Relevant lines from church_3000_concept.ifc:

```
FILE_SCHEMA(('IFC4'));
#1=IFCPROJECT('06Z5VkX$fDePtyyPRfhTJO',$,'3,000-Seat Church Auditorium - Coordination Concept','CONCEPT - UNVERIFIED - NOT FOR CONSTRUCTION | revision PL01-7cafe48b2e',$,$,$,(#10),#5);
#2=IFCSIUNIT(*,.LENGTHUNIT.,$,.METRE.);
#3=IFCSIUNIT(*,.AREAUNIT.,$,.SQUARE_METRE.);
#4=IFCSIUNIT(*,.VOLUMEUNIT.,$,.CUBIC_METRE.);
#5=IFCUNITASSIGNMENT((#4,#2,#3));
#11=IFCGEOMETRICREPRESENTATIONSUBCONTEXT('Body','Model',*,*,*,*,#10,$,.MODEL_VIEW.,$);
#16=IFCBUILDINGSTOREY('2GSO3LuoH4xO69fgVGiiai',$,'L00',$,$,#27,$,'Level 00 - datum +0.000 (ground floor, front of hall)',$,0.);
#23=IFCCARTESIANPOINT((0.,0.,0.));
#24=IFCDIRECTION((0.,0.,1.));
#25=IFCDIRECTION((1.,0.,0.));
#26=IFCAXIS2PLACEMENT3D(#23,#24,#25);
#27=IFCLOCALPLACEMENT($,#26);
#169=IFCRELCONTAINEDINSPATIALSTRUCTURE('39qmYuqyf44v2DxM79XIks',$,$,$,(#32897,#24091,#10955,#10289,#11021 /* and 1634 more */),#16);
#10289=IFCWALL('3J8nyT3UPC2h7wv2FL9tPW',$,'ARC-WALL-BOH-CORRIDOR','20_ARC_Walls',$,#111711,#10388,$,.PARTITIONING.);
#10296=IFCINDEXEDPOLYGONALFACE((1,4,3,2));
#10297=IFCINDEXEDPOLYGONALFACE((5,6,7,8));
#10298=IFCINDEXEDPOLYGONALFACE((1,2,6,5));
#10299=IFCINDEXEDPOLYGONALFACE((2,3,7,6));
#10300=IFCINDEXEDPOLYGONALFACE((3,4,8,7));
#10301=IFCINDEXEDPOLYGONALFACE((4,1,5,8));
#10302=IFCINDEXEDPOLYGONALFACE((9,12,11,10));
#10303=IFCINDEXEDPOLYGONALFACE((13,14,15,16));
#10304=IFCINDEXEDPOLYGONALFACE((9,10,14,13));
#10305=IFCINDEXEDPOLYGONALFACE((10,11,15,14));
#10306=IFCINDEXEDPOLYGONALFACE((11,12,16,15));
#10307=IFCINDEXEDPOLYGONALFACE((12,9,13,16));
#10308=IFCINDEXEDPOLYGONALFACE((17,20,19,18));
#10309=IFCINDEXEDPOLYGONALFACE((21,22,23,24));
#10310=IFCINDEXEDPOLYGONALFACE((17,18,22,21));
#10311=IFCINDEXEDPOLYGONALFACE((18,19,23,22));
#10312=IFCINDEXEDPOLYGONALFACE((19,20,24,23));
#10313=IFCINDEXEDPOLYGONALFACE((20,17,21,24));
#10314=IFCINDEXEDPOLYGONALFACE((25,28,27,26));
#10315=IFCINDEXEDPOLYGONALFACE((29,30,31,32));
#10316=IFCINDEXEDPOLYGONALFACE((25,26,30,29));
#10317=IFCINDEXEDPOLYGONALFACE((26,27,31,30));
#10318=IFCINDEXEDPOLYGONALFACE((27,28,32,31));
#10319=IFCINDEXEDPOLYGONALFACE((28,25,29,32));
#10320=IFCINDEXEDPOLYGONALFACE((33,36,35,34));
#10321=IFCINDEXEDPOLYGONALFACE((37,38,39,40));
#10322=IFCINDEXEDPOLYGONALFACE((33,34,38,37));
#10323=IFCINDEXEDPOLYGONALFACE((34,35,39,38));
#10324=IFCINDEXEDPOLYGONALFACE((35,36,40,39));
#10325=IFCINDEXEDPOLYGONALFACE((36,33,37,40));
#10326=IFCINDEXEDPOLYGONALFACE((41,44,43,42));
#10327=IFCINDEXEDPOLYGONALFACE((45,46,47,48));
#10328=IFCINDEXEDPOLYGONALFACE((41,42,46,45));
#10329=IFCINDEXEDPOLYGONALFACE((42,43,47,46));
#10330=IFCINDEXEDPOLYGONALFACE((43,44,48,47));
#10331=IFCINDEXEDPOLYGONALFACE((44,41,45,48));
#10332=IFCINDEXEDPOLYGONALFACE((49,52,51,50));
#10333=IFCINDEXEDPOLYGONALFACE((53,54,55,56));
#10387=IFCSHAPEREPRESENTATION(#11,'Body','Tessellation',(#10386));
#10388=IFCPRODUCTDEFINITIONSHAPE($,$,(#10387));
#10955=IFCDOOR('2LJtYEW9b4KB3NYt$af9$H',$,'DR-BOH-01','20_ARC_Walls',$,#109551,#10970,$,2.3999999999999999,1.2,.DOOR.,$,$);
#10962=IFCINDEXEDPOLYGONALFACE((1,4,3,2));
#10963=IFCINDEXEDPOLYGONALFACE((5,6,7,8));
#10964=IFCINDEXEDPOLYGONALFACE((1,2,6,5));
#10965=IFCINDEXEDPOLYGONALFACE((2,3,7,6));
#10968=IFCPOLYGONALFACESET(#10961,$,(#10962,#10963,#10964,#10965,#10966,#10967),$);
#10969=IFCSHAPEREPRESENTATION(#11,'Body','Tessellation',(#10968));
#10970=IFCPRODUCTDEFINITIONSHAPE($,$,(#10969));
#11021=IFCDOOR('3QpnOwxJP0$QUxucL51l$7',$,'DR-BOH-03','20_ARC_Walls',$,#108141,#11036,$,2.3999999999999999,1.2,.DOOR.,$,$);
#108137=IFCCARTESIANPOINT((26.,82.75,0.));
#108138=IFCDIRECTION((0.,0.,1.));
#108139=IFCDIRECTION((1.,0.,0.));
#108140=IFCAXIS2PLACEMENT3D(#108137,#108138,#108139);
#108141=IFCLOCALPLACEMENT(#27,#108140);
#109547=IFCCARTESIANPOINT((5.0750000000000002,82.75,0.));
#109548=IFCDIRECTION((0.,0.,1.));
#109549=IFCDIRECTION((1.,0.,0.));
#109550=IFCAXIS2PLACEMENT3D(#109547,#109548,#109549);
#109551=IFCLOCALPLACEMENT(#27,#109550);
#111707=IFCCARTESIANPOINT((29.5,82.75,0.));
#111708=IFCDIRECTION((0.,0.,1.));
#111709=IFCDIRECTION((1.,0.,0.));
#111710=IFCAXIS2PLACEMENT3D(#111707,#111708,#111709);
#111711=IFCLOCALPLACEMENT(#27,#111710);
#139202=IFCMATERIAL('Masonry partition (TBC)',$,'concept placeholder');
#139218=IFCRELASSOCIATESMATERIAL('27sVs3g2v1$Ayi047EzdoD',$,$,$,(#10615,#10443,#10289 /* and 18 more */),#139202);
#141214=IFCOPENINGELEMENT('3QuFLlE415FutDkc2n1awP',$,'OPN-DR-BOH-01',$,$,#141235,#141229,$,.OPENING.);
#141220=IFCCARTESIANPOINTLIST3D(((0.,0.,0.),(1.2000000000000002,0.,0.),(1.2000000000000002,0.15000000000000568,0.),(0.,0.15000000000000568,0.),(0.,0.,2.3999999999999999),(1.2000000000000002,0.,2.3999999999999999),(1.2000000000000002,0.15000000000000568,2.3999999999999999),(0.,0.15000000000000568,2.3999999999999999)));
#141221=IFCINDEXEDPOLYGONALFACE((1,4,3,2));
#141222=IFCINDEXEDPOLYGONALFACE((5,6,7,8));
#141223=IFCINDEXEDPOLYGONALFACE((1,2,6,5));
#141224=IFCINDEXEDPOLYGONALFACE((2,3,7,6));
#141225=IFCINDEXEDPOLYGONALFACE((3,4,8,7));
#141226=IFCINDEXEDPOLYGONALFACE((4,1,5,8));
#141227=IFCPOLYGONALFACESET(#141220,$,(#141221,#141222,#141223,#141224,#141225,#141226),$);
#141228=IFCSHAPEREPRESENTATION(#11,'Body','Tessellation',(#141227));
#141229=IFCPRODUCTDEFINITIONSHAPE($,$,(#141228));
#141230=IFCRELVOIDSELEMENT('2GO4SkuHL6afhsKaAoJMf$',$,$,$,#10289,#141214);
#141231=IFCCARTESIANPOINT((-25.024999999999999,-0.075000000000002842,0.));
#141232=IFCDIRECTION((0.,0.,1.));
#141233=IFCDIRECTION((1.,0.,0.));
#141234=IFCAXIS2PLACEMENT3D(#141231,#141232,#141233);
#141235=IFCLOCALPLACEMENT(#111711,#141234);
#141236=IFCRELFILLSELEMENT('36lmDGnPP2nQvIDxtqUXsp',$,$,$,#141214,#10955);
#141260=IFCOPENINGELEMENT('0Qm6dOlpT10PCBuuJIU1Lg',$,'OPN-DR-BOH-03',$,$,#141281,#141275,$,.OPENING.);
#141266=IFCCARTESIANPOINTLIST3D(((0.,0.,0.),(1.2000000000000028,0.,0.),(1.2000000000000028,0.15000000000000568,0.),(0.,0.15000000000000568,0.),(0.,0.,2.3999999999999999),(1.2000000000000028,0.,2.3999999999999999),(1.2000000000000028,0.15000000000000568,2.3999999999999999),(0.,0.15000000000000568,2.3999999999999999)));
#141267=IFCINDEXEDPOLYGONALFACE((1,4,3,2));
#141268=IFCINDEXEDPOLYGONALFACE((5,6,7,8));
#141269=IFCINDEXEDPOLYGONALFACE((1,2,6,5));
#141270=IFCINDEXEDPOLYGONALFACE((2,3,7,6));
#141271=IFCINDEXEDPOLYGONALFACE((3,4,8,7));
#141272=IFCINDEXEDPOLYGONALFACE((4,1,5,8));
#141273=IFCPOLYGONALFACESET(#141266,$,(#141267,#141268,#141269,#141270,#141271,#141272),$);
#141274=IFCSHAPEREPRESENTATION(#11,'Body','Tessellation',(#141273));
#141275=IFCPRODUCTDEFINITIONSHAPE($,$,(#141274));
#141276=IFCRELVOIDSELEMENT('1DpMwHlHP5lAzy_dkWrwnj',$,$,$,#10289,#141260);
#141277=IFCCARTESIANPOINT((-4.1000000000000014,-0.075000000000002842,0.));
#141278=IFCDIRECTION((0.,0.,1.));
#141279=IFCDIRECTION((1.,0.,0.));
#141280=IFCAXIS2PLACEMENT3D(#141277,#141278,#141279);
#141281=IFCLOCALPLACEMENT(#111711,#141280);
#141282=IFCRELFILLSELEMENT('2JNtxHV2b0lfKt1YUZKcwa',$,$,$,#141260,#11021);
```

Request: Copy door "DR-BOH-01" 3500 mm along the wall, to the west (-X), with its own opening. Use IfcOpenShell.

```python
import ifcopenshell
import ifcopenshell.api.feature
import ifcopenshell.api.geometry
import ifcopenshell.api.root
import ifcopenshell.geom
import ifcopenshell.util.element
import ifcopenshell.util.placement
import ifcopenshell.util.shape

model = ifcopenshell.open("church_3000_concept.ifc")
settings = ifcopenshell.geom.settings()


def volume(element):
    """Net volume in cubic metres, openings subtracted."""
    shape = ifcopenshell.geom.create_shape(settings, element)
    return ifcopenshell.util.shape.get_volume(shape.geometry)


door = model.by_guid("2LJtYEW9b4KB3NYt$af9$H")
opening = door.FillsVoids[0].RelatingOpeningElement
wall = opening.VoidsElements[0].RelatingBuildingElement
before = volume(wall)
shift = ifcopenshell.util.placement.get_local_placement(wall.ObjectPlacement)[:3, 0] * -3.5

# copy_class copies the void relationship, type, container and properties, but no geometry.
new_opening = ifcopenshell.api.root.copy_class(model, product=opening)
new_opening.Representation = ifcopenshell.util.element.copy_deep(
    model, opening.Representation, exclude=["IfcGeometricRepresentationContext", "IfcRepresentationMap"]
)
new_door = ifcopenshell.api.root.copy_class(model, product=door)
new_door.Representation = ifcopenshell.util.element.copy_deep(
    model, door.Representation, exclude=["IfcGeometricRepresentationContext", "IfcRepresentationMap"]
)
ifcopenshell.api.feature.add_filling(model, opening=new_opening, element=new_door)

for old, new in ((opening, new_opening), (door, new_door)):
    matrix = ifcopenshell.util.placement.get_local_placement(old.ObjectPlacement)
    matrix[:3, 3] += shift
    ifcopenshell.api.geometry.edit_object_placement(model, product=new, matrix=matrix, is_si=False)

after = volume(wall)

print(f"wall volume {before:.3f} -> {after:.3f} m3")

model.write("church_3000_concept_v2.ifc")
```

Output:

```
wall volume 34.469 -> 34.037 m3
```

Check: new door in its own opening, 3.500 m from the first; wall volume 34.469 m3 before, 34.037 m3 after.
